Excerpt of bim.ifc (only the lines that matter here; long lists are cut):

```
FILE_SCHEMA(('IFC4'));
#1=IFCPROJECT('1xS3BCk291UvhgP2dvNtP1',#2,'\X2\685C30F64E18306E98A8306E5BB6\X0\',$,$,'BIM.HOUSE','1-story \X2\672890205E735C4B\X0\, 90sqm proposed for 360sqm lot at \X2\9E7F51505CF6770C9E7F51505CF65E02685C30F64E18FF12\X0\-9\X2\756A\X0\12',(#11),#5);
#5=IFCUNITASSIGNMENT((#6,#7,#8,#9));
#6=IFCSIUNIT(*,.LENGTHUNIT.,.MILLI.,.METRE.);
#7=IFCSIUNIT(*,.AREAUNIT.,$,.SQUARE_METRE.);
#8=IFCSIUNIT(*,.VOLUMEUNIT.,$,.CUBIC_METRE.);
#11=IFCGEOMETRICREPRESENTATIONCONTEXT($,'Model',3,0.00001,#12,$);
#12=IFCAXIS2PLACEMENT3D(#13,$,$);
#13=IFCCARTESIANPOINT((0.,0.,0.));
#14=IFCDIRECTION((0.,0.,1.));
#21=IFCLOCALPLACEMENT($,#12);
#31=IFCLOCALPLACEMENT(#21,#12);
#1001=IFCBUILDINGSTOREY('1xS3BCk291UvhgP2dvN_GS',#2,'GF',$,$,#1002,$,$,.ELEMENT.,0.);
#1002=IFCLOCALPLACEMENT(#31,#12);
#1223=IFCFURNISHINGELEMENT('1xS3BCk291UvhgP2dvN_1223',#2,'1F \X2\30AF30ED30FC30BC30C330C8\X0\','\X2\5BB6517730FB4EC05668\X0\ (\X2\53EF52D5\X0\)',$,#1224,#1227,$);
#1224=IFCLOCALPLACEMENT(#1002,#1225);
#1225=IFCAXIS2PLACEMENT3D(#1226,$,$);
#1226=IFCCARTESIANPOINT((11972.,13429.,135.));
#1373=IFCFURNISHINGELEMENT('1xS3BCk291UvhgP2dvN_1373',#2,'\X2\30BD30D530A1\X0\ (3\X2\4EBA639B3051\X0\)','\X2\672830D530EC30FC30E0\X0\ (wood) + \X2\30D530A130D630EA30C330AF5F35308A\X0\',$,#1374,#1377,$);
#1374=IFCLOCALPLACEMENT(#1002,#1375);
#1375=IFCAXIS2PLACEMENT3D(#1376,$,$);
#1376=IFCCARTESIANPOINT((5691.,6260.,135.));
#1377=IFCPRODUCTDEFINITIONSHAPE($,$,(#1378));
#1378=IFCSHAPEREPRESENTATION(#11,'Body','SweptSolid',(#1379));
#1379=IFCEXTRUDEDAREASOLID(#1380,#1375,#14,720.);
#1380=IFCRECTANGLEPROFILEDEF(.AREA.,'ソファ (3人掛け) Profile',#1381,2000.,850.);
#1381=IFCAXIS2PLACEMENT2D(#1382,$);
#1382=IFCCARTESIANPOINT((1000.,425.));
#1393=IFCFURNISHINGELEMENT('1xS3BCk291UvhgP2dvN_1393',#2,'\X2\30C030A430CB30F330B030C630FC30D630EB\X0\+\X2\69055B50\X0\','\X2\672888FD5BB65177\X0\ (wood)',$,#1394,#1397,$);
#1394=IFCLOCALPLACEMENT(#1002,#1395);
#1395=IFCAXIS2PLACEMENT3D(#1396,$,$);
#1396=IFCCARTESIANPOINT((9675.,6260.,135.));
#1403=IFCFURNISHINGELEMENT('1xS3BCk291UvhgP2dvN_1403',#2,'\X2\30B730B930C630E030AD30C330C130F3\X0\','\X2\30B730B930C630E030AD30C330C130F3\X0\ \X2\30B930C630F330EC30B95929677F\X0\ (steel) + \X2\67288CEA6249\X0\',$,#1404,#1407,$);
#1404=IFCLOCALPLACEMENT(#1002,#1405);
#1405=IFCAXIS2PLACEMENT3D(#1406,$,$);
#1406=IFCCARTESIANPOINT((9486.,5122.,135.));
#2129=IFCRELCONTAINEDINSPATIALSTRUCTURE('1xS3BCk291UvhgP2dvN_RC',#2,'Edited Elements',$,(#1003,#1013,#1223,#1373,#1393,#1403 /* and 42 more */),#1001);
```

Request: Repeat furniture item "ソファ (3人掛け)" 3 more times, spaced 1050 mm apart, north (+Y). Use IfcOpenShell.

```python
import numpy as np
import ifcopenshell
import ifcopenshell.api.geometry
import ifcopenshell.api.root
import ifcopenshell.util.element
import ifcopenshell.util.placement

model = ifcopenshell.open("bim.ifc")


def reuse_history(source, copy):
    """copy_class also copies each property set's owner history, people and application; keep the originals."""
    for rel in copy.IsDefinedBy:
        if rel.is_a("IfcRelDefinesByProperties") and (history := rel.RelatingPropertyDefinition.OwnerHistory):
            rel.RelatingPropertyDefinition.OwnerHistory = source.OwnerHistory
            ifcopenshell.util.element.remove_deep2(model, history)


source = model.by_id(1373)
base = ifcopenshell.util.placement.get_local_placement(source.ObjectPlacement)
step = np.array([0.0, 1.0, 0.0]) * 1050.0

for i in range(1, 4):
    copy = ifcopenshell.api.root.copy_class(model, product=source)
    copy.Representation = ifcopenshell.util.element.copy_deep(
        model, source.Representation, exclude=["IfcGeometricRepresentationContext", "IfcRepresentationMap"]
    )
    reuse_history(source, copy)
    matrix = base.copy()
    matrix[:3, 3] += i * step
    print("added at", matrix[:3, 3].round(3) + 0.0)
    ifcopenshell.api.geometry.edit_object_placement(model, product=copy, matrix=matrix, is_si=False)

model.write("bim_v2.ifc")
```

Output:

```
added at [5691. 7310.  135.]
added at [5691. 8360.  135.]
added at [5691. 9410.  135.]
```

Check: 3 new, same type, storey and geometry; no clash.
